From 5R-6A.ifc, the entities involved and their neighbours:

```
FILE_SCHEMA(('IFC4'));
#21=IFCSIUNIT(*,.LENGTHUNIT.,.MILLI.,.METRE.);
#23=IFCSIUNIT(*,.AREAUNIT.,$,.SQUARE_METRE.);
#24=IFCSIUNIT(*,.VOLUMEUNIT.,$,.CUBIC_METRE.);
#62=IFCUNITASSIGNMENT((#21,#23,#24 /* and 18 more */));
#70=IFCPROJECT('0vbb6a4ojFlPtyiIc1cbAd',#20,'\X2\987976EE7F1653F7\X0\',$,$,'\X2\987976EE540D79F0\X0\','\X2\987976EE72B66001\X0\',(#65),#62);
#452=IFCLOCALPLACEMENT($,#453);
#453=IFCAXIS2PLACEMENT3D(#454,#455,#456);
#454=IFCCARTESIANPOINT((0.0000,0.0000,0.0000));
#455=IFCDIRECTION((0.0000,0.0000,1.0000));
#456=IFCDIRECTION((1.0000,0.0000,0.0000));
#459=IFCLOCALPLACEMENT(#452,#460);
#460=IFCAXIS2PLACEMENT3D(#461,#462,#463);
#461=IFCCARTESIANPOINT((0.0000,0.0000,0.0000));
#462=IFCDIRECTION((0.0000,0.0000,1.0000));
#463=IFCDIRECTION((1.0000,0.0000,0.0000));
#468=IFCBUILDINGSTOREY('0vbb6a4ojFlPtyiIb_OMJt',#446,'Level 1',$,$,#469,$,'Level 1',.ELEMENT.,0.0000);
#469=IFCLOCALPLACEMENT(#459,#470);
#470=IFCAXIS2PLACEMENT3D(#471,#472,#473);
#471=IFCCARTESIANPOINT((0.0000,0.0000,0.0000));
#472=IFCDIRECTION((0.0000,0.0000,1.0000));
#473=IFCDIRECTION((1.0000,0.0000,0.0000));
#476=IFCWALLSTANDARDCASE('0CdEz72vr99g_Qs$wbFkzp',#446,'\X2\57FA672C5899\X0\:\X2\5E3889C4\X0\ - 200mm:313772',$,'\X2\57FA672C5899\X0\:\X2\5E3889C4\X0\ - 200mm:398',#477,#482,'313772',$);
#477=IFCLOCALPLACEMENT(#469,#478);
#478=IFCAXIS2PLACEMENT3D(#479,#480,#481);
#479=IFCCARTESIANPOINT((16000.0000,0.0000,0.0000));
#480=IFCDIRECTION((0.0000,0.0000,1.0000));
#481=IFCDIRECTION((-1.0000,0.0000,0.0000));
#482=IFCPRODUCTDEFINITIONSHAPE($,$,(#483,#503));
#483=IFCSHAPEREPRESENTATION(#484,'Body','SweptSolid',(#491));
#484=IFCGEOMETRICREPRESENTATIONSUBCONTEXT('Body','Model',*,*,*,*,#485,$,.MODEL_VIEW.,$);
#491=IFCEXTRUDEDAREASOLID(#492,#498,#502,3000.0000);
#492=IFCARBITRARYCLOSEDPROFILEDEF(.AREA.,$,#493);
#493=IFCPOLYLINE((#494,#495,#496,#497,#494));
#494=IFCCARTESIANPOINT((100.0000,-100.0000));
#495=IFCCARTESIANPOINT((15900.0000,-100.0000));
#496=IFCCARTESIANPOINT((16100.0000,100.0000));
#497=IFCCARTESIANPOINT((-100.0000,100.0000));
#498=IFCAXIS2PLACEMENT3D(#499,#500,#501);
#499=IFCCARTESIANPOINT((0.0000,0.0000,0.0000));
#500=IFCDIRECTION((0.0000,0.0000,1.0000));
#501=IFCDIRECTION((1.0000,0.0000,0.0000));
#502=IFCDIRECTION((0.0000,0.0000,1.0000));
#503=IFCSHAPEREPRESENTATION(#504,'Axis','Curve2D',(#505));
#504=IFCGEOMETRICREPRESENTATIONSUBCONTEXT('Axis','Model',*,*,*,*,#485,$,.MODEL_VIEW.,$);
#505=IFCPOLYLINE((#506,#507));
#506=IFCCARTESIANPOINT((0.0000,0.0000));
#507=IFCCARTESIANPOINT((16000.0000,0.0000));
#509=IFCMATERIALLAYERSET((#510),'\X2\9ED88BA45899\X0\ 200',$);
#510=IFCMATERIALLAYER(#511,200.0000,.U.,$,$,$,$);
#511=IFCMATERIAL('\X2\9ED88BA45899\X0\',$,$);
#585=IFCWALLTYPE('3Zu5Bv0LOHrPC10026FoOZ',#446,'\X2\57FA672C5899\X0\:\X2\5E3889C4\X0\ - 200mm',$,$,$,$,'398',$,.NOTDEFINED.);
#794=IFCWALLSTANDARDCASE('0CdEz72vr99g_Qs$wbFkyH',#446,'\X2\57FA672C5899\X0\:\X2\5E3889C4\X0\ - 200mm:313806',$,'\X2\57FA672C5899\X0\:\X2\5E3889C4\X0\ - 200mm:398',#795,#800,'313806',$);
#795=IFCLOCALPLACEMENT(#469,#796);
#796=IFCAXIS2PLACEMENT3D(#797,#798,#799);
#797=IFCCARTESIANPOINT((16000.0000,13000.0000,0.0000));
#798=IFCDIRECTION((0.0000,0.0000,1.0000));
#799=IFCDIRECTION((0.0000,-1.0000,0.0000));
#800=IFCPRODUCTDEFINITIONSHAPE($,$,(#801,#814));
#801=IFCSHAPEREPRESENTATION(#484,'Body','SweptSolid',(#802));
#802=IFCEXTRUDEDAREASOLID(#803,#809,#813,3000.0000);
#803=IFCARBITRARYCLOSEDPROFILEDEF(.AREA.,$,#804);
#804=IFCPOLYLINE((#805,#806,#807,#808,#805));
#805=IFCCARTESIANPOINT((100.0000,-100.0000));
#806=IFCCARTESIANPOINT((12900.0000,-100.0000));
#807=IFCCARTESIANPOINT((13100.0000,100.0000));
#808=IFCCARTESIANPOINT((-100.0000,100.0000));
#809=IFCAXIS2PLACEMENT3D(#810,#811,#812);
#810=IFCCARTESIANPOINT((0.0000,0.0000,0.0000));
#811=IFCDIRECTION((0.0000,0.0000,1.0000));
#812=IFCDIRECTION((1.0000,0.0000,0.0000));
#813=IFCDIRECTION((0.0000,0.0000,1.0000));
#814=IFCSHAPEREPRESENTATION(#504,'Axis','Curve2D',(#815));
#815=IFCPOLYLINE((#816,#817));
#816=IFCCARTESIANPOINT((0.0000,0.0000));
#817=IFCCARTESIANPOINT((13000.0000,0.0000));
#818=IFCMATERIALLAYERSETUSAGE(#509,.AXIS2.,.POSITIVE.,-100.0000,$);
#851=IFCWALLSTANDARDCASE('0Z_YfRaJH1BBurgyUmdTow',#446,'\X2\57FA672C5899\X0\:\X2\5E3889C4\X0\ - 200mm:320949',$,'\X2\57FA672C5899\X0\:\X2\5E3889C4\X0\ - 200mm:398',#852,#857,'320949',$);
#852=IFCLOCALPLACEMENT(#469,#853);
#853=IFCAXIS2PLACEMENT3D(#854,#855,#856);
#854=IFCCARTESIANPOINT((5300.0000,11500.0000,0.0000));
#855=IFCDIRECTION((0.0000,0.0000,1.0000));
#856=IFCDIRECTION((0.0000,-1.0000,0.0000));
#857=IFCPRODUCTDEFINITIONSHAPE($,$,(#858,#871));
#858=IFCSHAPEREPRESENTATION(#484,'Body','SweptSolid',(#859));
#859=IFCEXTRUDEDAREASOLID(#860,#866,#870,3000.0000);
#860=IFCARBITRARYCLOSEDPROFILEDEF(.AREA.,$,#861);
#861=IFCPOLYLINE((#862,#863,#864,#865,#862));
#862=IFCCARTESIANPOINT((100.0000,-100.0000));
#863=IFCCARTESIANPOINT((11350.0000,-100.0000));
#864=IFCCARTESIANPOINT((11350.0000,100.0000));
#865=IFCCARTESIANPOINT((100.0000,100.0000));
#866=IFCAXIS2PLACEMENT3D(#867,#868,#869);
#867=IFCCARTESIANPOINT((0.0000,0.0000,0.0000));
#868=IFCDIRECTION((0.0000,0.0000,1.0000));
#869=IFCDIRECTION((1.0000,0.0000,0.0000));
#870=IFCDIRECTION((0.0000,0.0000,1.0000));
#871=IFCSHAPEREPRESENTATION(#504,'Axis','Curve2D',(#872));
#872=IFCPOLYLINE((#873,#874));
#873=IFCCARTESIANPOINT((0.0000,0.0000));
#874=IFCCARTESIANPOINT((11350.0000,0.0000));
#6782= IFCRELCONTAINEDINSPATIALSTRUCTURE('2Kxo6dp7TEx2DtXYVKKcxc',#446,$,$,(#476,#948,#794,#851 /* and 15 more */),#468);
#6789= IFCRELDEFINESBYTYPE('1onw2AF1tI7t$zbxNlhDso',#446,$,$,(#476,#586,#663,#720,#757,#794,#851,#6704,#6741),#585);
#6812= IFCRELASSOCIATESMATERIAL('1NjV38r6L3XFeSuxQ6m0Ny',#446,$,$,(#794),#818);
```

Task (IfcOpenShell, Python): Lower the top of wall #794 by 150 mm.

```python
import ifcopenshell
import ifcopenshell.geom
import ifcopenshell.util.representation
import ifcopenshell.util.shape
import ifcopenshell.util.unit

model = ifcopenshell.open("5R-6A.ifc")
unit_scale = ifcopenshell.util.unit.calculate_unit_scale(model)
settings = ifcopenshell.geom.settings()


def volume(element):
    """Net volume in cubic metres, openings subtracted."""
    shape = ifcopenshell.geom.create_shape(settings, element)
    return ifcopenshell.util.shape.get_volume(shape.geometry)


wall = model.by_guid("0CdEz72vr99g_Qs$wbFkyH")
before = volume(wall)

body = ifcopenshell.util.representation.get_representation(wall, "Model", "Body")
solid = body.Items[0]
old_height = solid.Depth
solid.Depth -= 0.15 / unit_scale
after = volume(wall)

print(f"height {old_height:g} -> {solid.Depth:g}, volume {before:.3f} -> {after:.3f} m3")

model.write("5R-6A-out.ifc")
```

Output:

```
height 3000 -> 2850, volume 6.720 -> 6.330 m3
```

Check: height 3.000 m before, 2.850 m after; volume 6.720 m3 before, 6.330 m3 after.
